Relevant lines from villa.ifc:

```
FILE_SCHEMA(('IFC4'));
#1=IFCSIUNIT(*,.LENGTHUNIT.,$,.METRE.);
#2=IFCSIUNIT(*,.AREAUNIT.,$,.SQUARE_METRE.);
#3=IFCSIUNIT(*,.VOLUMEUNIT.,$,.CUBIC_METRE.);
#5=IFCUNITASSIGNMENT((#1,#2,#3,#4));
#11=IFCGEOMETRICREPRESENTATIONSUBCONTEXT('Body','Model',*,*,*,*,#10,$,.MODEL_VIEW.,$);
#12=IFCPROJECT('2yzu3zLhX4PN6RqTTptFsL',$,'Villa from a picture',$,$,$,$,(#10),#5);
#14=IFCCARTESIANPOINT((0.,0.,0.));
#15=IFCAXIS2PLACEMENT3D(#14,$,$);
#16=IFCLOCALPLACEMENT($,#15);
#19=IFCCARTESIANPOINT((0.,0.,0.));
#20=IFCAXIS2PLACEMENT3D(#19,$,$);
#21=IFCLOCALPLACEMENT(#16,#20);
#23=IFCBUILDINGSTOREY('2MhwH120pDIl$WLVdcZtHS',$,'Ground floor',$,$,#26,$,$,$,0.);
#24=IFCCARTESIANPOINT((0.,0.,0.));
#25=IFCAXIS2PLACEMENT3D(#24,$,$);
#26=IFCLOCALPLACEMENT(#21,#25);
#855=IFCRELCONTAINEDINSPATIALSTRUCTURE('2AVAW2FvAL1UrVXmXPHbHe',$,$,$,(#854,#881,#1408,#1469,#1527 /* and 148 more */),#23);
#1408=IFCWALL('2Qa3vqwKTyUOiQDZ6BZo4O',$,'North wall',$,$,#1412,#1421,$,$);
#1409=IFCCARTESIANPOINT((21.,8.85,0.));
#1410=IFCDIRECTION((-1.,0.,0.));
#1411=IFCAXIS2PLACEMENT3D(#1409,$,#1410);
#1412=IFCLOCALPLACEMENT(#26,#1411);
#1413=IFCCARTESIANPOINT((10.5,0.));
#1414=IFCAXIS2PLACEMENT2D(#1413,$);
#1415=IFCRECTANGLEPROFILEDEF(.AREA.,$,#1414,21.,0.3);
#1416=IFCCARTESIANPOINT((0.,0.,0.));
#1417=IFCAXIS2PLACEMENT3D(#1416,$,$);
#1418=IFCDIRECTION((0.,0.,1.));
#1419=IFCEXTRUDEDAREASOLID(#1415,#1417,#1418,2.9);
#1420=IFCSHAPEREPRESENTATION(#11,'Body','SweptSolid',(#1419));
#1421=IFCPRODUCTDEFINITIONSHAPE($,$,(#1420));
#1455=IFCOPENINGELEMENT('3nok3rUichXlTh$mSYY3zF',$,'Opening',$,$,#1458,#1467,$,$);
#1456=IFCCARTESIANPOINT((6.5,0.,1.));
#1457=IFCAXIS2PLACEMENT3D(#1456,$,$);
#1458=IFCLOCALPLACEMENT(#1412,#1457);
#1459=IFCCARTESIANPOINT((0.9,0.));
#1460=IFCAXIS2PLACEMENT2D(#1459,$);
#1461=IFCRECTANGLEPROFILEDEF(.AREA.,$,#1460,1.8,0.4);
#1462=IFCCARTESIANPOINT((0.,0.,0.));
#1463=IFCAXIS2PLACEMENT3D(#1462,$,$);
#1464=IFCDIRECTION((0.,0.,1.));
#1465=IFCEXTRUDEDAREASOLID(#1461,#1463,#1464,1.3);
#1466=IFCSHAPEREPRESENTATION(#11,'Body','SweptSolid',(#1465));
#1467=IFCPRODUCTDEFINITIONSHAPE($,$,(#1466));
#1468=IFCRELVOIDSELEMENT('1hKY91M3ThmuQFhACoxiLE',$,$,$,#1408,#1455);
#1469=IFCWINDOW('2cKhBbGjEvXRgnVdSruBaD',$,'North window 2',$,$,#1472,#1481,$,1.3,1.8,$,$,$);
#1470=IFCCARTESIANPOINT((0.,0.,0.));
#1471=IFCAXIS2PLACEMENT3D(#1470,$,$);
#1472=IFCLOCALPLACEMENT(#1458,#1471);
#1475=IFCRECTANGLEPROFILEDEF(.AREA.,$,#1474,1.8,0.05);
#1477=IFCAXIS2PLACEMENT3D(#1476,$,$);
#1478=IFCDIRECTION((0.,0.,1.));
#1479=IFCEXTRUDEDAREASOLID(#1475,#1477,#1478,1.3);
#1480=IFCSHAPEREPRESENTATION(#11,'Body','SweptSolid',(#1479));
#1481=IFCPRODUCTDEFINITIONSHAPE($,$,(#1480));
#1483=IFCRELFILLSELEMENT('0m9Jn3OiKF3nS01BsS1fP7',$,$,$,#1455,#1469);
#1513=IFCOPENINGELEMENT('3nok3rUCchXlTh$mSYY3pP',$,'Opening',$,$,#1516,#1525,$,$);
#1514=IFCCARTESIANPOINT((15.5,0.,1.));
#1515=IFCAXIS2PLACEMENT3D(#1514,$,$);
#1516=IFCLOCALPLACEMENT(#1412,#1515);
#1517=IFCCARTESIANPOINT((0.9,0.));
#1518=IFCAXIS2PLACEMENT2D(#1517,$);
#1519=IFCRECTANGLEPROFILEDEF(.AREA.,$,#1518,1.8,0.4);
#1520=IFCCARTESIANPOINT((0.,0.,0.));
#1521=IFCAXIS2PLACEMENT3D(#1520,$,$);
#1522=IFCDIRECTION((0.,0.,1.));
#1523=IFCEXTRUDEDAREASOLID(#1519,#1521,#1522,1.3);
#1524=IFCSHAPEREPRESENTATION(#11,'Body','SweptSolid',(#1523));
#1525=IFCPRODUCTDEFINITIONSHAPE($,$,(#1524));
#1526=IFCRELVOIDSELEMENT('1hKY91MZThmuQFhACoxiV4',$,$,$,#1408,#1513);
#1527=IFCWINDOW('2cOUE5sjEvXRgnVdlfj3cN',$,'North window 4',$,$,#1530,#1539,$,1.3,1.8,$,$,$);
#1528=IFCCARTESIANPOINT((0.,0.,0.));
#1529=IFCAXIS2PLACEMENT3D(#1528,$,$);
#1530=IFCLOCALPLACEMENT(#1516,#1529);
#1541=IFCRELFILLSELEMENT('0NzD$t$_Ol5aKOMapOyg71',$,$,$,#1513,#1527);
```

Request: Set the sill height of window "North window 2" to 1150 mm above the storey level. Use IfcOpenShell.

```python
import numpy as np
import ifcopenshell
import ifcopenshell.api.geometry
import ifcopenshell.geom
import ifcopenshell.util.element
import ifcopenshell.util.placement
import ifcopenshell.util.shape
import ifcopenshell.util.unit

model = ifcopenshell.open("villa.ifc")
unit_scale = ifcopenshell.util.unit.calculate_unit_scale(model)

window = model.by_guid("2cKhBbGjEvXRgnVdSruBaD")
opening = window.FillsVoids[0].RelatingOpeningElement
storey = ifcopenshell.util.element.get_container(window, ifc_class="IfcBuildingStorey")
level = ifcopenshell.util.placement.get_local_placement(storey.ObjectPlacement)[2, 3]

# The opening's origin need not be at the sill, so measure its lowest point.
shape = ifcopenshell.geom.create_shape(ifcopenshell.geom.settings(), opening)
bottom = ifcopenshell.util.shape.get_shape_bottom_elevation(shape, shape.geometry) / unit_scale
dz = level + 1.15 / unit_scale - bottom

shift = np.array([0.0, 0.0, dz])
# The window is placed relative to its opening, so it follows when the opening moves.
matrix = ifcopenshell.util.placement.get_local_placement(opening.ObjectPlacement)
matrix[:3, 3] += shift
ifcopenshell.api.geometry.edit_object_placement(
    model, product=opening, matrix=matrix, is_si=False, should_transform_children=True
)

print(f"moved by {dz * unit_scale:+.3f} m")

model.write("villa_rev.ifc")
```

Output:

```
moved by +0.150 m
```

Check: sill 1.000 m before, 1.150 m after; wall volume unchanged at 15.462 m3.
